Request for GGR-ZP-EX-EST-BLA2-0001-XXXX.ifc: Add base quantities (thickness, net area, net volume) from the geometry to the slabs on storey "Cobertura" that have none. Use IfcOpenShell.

First a look at what the model holds.

```python
import ifcopenshell
import ifcopenshell.util.element
import ifcopenshell.util.unit

model = ifcopenshell.open("GGR-ZP-EX-EST-BLA2-0001-XXXX.ifc")
print(model.schema)
for unit_type in ("LENGTHUNIT", "AREAUNIT", "VOLUMEUNIT"):
    print(unit_type, ifcopenshell.util.unit.calculate_unit_scale(model, unit_type))
storey = next(s for s in model.by_type("IfcBuildingStorey") if s.Name == "Cobertura")
slabs = [e for e in ifcopenshell.util.element.get_decomposition(storey) if e.is_a("IfcSlab")]
for e in sorted(slabs, key=lambda e: e.id()):
    print(e.id(), e.is_a(), e.Name, list(ifcopenshell.util.element.get_psets(e, qtos_only=True)), sep=" | ")
```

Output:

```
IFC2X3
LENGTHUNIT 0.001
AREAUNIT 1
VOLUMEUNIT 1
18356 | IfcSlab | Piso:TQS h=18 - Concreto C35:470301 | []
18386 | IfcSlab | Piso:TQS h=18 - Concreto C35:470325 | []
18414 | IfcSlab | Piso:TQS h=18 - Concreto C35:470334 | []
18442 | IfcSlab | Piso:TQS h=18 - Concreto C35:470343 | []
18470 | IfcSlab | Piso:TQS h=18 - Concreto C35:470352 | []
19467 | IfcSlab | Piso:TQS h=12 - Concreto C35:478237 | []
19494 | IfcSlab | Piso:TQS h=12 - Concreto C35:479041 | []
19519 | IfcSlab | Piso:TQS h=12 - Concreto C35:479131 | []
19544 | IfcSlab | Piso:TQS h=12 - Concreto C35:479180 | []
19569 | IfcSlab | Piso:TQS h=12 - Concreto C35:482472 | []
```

```python
import ifcopenshell
import ifcopenshell.api.pset
import ifcopenshell.geom
import ifcopenshell.util.element
import ifcopenshell.util.shape
import ifcopenshell.util.unit

model = ifcopenshell.open("GGR-ZP-EX-EST-BLA2-0001-XXXX.ifc")
unit_scale = ifcopenshell.util.unit.calculate_unit_scale(model)
area_scale = ifcopenshell.util.unit.calculate_unit_scale(model, "AREAUNIT")
volume_scale = ifcopenshell.util.unit.calculate_unit_scale(model, "VOLUMEUNIT")
settings = ifcopenshell.geom.settings()

storey = next(s for s in model.by_type("IfcBuildingStorey") if s.Name == "Cobertura")
slabs = [e for e in ifcopenshell.util.element.get_decomposition(storey) if e.is_a("IfcSlab")]

for e in sorted(slabs, key=lambda e: e.id()):
    if ifcopenshell.util.element.get_psets(e, qtos_only=True, should_inherit=False):
        continue
    # Geometry comes back in metres, in the element's own axes.
    shape = ifcopenshell.geom.create_shape(settings, e)
    values = {
        "Width": ifcopenshell.util.shape.get_z(shape.geometry) / unit_scale,
        "NetArea": ifcopenshell.util.shape.get_footprint_area(shape.geometry) / area_scale,
        "NetVolume": ifcopenshell.util.shape.get_volume(shape.geometry) / volume_scale,
    }
    qto = ifcopenshell.api.pset.add_qto(model, product=e, name="BaseQuantities")
    ifcopenshell.api.pset.edit_qto(model, qto=qto, properties=values)
    print(e.id(), {k: round(v, 3) for k, v in values.items()})

model.write("GGR-ZP-EX-EST-BLA2-0001-XXXX_updated.ifc")
```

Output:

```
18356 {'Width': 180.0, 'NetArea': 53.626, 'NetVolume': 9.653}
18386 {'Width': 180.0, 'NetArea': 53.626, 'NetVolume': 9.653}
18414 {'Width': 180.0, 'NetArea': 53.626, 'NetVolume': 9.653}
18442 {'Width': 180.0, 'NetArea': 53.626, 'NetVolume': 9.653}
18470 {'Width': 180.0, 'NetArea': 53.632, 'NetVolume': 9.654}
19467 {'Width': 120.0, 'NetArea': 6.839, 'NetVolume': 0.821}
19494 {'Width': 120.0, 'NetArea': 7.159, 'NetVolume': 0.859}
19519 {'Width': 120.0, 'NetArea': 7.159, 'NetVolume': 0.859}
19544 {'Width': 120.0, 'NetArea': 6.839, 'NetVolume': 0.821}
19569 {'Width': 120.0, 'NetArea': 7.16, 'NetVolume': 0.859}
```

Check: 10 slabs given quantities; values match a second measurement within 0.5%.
